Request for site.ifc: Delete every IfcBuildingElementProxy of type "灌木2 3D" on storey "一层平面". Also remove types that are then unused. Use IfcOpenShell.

First a look at what the model holds.

```python
import ifcopenshell
import ifcopenshell.util.element

model = ifcopenshell.open("site.ifc")
print(model.schema)
storey = next(s for s in model.by_type("IfcBuildingStorey") if s.Name == "一层平面")
proxies = [e for e in ifcopenshell.util.element.get_decomposition(storey) if e.is_a("IfcBuildingElementProxy")]
seen = {}
for e in proxies:
    element_type = ifcopenshell.util.element.get_type(e)
    name = element_type.Name if element_type not in (None, e) else None
    seen[name] = seen.get(name, 0) + 1
for name, count in sorted(seen.items(), key=str):
    print(count, "x", name)
```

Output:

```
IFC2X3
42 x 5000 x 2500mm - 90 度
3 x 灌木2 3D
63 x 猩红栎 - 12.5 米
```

```python
import ifcopenshell
import ifcopenshell.api.root
import ifcopenshell.util.element

model = ifcopenshell.open("site.ifc")

storey = next(s for s in model.by_type("IfcBuildingStorey") if s.Name == "一层平面")
proxies = [e for e in ifcopenshell.util.element.get_decomposition(storey) if e.is_a("IfcBuildingElementProxy")]
targets = [e for e in proxies if (t := ifcopenshell.util.element.get_type(e)) not in (None, e) and t.Name == "灌木2 3D"]
types = {ifcopenshell.util.element.get_type(e) for e in targets} - {None, *targets}

for e in targets:
    ifcopenshell.api.root.remove_product(model, product=e)
print(len(targets), "removed")

unused = [t for t in types if not ifcopenshell.util.element.get_types(t)]
for t in unused:
    ifcopenshell.api.root.remove_product(model, product=t)
print(len(unused), "unused types removed")

model.write("site_rev.ifc")
```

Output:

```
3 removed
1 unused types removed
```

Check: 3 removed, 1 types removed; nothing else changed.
